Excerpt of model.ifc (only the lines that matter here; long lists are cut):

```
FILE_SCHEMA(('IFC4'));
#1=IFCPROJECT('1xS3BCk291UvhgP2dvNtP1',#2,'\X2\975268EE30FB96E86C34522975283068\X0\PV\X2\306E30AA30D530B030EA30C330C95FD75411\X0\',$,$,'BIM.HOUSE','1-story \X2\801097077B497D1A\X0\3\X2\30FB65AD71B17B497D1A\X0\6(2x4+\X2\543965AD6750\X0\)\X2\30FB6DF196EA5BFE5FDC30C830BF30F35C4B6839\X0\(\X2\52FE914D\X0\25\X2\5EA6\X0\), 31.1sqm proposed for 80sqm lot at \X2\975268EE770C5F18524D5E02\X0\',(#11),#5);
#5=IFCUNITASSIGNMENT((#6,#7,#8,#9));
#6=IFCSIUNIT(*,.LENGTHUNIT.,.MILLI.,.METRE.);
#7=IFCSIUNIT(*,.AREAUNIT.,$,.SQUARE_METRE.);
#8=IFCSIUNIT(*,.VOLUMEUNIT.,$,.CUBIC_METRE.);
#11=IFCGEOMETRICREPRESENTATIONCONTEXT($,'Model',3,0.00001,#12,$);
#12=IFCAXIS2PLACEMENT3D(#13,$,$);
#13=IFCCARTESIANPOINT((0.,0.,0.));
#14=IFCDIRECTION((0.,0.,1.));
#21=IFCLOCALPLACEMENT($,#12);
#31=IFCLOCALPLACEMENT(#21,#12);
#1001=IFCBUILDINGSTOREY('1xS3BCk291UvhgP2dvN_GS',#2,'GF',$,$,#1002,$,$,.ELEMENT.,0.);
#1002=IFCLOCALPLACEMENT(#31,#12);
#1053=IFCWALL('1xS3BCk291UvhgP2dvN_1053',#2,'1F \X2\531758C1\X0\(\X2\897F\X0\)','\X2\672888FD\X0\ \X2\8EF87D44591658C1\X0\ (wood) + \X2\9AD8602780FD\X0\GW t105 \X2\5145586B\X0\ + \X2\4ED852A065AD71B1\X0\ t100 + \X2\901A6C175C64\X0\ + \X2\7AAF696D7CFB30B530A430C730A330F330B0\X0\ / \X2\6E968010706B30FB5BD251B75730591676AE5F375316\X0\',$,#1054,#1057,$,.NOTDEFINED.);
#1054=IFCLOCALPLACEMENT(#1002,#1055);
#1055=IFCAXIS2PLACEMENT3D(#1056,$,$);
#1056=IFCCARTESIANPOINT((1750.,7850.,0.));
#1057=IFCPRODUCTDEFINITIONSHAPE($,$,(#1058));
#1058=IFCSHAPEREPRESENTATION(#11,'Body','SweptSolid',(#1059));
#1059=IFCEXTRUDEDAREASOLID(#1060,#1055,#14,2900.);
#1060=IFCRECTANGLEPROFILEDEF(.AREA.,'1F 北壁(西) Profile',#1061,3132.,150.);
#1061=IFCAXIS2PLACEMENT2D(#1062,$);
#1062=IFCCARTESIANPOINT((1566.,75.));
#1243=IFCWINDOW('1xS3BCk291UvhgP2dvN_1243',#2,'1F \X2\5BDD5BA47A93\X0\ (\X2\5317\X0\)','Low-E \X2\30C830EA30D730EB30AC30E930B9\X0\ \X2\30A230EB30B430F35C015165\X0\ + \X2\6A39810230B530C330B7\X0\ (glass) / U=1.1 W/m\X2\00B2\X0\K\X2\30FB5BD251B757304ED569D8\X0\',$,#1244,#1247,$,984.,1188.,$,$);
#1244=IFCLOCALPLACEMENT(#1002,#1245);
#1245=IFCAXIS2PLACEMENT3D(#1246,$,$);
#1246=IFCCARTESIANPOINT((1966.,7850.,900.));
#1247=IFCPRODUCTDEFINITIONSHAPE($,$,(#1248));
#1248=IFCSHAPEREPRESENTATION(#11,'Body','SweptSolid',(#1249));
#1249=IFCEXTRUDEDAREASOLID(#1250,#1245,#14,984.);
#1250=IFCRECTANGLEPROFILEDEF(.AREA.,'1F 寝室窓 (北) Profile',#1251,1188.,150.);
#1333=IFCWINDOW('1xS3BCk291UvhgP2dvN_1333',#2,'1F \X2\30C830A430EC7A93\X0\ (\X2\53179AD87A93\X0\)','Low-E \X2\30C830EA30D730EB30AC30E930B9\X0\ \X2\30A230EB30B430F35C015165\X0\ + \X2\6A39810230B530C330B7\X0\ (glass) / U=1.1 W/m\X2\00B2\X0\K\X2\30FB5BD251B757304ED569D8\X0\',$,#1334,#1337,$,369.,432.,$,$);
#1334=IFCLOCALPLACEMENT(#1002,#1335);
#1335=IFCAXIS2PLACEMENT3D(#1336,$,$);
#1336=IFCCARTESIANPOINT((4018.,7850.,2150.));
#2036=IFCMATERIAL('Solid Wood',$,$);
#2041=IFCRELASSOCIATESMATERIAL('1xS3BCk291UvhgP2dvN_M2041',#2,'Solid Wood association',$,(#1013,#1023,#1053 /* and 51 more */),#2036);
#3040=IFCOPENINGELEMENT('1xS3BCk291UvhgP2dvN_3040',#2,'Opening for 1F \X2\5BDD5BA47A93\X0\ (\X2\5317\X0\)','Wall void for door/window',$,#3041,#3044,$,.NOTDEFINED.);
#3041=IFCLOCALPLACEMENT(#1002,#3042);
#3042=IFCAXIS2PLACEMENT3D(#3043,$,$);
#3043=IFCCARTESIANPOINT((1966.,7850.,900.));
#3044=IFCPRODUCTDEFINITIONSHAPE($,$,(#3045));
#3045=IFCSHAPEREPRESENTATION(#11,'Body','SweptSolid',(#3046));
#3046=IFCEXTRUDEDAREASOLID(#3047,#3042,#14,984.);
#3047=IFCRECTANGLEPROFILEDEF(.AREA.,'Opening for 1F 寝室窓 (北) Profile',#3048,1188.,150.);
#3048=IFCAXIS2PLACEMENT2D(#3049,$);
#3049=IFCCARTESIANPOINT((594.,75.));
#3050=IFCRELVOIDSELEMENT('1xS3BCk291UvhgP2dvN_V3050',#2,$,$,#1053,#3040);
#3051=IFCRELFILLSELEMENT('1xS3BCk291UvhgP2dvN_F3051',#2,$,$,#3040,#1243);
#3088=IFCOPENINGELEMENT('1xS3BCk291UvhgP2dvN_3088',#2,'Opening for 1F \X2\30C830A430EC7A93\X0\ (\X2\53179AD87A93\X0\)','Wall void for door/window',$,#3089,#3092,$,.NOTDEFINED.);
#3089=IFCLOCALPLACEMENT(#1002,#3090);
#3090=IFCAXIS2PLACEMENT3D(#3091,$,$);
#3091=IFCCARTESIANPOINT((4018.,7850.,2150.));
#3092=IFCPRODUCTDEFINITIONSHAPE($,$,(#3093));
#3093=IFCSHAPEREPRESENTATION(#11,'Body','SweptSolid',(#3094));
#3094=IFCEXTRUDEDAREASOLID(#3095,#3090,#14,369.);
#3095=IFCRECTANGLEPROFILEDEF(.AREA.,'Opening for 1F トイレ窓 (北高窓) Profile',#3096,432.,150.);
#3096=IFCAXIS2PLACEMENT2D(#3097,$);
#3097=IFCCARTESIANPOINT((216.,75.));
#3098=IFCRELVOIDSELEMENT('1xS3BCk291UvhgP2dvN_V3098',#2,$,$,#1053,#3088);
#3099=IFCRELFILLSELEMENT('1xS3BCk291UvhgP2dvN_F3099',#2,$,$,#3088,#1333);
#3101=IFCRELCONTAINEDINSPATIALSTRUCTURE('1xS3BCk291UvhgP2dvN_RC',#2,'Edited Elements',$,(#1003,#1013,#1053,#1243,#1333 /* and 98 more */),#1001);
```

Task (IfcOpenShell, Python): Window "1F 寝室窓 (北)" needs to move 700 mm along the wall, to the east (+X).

```python
import ifcopenshell
import ifcopenshell.api.geometry
import ifcopenshell.util.placement
import ifcopenshell.util.unit

model = ifcopenshell.open("model.ifc")
unit_scale = ifcopenshell.util.unit.calculate_unit_scale(model)

window = model.by_id(1243)
opening = window.FillsVoids[0].RelatingOpeningElement
wall = opening.VoidsElements[0].RelatingBuildingElement

wall_matrix = ifcopenshell.util.placement.get_local_placement(wall.ObjectPlacement)
shift = wall_matrix[:3, 0] * 0.7 / unit_scale
before = ifcopenshell.util.placement.get_local_placement(window.ObjectPlacement)[:3, 3].copy()

# The window is not placed relative to its opening, so move both.
for product in (opening, window):
    matrix = ifcopenshell.util.placement.get_local_placement(product.ObjectPlacement)
    matrix[:3, 3] += shift
    ifcopenshell.api.geometry.edit_object_placement(model, product=product, matrix=matrix, is_si=False)

after = ifcopenshell.util.placement.get_local_placement(window.ObjectPlacement)[:3, 3]
print("window moved by", (after - before).round(3) + 0.0)

model.write("model_rev.ifc")
```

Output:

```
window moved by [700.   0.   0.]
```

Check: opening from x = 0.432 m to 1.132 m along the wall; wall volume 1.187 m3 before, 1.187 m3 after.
